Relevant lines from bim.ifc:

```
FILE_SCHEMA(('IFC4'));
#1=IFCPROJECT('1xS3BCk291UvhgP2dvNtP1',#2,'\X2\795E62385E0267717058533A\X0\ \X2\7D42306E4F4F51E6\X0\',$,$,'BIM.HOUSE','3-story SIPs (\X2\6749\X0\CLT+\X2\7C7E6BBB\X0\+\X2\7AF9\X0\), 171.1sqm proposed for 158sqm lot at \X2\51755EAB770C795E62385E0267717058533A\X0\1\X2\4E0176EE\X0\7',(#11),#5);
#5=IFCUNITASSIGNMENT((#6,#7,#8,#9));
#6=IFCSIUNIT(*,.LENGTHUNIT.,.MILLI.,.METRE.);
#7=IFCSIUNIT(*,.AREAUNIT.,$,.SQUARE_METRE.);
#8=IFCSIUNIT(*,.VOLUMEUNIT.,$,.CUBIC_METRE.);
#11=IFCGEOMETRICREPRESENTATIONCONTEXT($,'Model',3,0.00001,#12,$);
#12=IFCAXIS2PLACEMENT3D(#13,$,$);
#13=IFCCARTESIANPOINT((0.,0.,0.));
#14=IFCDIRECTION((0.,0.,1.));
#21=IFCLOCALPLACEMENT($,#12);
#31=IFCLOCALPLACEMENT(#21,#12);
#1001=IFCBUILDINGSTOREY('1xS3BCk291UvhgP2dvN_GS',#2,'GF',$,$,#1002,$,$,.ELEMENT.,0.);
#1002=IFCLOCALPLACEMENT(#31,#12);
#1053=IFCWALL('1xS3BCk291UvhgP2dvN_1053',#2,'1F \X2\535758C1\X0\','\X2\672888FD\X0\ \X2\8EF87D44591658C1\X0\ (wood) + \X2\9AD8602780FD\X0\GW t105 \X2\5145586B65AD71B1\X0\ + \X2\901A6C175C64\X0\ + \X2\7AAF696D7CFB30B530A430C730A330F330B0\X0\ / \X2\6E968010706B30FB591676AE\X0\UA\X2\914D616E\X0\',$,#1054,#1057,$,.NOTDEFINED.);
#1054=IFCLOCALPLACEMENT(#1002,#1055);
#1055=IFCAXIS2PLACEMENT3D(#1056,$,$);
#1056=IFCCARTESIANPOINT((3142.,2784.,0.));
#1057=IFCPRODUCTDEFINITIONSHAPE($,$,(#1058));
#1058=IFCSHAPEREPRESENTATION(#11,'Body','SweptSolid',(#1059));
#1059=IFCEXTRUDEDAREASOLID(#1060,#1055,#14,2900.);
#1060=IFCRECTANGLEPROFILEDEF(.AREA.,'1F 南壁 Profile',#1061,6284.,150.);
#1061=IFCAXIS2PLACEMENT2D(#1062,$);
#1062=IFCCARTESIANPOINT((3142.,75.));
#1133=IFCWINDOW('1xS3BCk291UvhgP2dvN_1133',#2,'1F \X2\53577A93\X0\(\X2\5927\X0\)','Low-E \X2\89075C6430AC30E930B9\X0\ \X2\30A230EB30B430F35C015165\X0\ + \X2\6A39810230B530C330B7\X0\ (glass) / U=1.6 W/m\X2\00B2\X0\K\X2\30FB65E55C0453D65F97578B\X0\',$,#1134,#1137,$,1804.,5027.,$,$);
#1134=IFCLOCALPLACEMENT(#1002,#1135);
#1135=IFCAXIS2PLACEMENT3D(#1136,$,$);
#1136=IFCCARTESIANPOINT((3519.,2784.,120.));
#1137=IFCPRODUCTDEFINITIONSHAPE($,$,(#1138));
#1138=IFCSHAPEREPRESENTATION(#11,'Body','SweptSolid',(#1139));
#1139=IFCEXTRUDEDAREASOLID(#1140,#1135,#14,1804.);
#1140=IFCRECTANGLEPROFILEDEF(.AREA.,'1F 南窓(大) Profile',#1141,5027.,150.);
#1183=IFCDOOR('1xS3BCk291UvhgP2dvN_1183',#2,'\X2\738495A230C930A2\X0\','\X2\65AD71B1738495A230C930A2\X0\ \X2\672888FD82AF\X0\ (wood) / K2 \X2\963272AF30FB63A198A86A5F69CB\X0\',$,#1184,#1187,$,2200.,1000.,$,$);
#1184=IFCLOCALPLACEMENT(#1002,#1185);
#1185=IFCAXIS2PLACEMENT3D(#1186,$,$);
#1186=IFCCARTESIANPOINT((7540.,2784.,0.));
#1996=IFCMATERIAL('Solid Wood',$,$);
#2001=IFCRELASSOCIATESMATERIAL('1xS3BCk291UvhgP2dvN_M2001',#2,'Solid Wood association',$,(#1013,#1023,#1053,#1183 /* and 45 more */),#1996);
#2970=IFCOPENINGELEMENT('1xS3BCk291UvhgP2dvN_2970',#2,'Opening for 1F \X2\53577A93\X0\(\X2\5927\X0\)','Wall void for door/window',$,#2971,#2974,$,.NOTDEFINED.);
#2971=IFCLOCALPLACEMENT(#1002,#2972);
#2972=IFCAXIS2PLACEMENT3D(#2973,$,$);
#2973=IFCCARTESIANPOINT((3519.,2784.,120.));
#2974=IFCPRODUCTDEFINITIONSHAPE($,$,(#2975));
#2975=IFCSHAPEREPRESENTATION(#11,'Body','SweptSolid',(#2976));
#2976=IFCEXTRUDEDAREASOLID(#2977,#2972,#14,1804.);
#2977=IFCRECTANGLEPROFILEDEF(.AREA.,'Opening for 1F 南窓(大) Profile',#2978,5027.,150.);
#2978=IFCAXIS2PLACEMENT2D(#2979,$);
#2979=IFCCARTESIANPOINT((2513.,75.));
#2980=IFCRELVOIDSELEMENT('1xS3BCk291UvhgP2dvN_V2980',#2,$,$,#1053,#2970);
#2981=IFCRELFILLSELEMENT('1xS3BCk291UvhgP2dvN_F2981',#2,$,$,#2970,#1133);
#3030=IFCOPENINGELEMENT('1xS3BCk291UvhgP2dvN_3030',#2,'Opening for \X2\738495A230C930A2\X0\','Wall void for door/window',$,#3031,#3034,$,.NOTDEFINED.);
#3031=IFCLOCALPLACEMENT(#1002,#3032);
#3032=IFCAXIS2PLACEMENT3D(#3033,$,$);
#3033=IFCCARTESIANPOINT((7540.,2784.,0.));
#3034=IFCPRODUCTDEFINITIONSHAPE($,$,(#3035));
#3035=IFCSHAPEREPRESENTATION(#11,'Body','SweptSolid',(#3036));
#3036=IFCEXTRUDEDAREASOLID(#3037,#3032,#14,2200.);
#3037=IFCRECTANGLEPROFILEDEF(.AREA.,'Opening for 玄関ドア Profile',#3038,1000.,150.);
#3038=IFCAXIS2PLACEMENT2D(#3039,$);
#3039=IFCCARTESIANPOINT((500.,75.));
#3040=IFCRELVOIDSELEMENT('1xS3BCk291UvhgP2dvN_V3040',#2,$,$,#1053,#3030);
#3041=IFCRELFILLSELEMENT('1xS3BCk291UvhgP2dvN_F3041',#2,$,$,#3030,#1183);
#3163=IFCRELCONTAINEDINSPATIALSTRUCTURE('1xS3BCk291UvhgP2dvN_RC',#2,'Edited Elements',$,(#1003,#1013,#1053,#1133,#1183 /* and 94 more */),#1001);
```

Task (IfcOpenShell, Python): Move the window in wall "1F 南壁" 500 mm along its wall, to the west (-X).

```python
import ifcopenshell
import ifcopenshell.api.geometry
import ifcopenshell.util.placement
import ifcopenshell.util.unit

model = ifcopenshell.open("bim.ifc")
unit_scale = ifcopenshell.util.unit.calculate_unit_scale(model)

window = model.by_guid("1xS3BCk291UvhgP2dvN_1133")
opening = window.FillsVoids[0].RelatingOpeningElement
wall = opening.VoidsElements[0].RelatingBuildingElement

wall_matrix = ifcopenshell.util.placement.get_local_placement(wall.ObjectPlacement)
shift = wall_matrix[:3, 0] * -0.5 / unit_scale
before = ifcopenshell.util.placement.get_local_placement(window.ObjectPlacement)[:3, 3].copy()

# The window is not placed relative to its opening, so move both.
for product in (opening, window):
    matrix = ifcopenshell.util.placement.get_local_placement(product.ObjectPlacement)
    matrix[:3, 3] += shift
    ifcopenshell.api.geometry.edit_object_placement(model, product=product, matrix=matrix, is_si=False)

after = ifcopenshell.util.placement.get_local_placement(window.ObjectPlacement)[:3, 3]
print("window moved by", (after - before).round(3) + 0.0)

model.write("bim_updated.ifc")
```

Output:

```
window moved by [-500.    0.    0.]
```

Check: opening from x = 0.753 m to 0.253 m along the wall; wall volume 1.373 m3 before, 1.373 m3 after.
